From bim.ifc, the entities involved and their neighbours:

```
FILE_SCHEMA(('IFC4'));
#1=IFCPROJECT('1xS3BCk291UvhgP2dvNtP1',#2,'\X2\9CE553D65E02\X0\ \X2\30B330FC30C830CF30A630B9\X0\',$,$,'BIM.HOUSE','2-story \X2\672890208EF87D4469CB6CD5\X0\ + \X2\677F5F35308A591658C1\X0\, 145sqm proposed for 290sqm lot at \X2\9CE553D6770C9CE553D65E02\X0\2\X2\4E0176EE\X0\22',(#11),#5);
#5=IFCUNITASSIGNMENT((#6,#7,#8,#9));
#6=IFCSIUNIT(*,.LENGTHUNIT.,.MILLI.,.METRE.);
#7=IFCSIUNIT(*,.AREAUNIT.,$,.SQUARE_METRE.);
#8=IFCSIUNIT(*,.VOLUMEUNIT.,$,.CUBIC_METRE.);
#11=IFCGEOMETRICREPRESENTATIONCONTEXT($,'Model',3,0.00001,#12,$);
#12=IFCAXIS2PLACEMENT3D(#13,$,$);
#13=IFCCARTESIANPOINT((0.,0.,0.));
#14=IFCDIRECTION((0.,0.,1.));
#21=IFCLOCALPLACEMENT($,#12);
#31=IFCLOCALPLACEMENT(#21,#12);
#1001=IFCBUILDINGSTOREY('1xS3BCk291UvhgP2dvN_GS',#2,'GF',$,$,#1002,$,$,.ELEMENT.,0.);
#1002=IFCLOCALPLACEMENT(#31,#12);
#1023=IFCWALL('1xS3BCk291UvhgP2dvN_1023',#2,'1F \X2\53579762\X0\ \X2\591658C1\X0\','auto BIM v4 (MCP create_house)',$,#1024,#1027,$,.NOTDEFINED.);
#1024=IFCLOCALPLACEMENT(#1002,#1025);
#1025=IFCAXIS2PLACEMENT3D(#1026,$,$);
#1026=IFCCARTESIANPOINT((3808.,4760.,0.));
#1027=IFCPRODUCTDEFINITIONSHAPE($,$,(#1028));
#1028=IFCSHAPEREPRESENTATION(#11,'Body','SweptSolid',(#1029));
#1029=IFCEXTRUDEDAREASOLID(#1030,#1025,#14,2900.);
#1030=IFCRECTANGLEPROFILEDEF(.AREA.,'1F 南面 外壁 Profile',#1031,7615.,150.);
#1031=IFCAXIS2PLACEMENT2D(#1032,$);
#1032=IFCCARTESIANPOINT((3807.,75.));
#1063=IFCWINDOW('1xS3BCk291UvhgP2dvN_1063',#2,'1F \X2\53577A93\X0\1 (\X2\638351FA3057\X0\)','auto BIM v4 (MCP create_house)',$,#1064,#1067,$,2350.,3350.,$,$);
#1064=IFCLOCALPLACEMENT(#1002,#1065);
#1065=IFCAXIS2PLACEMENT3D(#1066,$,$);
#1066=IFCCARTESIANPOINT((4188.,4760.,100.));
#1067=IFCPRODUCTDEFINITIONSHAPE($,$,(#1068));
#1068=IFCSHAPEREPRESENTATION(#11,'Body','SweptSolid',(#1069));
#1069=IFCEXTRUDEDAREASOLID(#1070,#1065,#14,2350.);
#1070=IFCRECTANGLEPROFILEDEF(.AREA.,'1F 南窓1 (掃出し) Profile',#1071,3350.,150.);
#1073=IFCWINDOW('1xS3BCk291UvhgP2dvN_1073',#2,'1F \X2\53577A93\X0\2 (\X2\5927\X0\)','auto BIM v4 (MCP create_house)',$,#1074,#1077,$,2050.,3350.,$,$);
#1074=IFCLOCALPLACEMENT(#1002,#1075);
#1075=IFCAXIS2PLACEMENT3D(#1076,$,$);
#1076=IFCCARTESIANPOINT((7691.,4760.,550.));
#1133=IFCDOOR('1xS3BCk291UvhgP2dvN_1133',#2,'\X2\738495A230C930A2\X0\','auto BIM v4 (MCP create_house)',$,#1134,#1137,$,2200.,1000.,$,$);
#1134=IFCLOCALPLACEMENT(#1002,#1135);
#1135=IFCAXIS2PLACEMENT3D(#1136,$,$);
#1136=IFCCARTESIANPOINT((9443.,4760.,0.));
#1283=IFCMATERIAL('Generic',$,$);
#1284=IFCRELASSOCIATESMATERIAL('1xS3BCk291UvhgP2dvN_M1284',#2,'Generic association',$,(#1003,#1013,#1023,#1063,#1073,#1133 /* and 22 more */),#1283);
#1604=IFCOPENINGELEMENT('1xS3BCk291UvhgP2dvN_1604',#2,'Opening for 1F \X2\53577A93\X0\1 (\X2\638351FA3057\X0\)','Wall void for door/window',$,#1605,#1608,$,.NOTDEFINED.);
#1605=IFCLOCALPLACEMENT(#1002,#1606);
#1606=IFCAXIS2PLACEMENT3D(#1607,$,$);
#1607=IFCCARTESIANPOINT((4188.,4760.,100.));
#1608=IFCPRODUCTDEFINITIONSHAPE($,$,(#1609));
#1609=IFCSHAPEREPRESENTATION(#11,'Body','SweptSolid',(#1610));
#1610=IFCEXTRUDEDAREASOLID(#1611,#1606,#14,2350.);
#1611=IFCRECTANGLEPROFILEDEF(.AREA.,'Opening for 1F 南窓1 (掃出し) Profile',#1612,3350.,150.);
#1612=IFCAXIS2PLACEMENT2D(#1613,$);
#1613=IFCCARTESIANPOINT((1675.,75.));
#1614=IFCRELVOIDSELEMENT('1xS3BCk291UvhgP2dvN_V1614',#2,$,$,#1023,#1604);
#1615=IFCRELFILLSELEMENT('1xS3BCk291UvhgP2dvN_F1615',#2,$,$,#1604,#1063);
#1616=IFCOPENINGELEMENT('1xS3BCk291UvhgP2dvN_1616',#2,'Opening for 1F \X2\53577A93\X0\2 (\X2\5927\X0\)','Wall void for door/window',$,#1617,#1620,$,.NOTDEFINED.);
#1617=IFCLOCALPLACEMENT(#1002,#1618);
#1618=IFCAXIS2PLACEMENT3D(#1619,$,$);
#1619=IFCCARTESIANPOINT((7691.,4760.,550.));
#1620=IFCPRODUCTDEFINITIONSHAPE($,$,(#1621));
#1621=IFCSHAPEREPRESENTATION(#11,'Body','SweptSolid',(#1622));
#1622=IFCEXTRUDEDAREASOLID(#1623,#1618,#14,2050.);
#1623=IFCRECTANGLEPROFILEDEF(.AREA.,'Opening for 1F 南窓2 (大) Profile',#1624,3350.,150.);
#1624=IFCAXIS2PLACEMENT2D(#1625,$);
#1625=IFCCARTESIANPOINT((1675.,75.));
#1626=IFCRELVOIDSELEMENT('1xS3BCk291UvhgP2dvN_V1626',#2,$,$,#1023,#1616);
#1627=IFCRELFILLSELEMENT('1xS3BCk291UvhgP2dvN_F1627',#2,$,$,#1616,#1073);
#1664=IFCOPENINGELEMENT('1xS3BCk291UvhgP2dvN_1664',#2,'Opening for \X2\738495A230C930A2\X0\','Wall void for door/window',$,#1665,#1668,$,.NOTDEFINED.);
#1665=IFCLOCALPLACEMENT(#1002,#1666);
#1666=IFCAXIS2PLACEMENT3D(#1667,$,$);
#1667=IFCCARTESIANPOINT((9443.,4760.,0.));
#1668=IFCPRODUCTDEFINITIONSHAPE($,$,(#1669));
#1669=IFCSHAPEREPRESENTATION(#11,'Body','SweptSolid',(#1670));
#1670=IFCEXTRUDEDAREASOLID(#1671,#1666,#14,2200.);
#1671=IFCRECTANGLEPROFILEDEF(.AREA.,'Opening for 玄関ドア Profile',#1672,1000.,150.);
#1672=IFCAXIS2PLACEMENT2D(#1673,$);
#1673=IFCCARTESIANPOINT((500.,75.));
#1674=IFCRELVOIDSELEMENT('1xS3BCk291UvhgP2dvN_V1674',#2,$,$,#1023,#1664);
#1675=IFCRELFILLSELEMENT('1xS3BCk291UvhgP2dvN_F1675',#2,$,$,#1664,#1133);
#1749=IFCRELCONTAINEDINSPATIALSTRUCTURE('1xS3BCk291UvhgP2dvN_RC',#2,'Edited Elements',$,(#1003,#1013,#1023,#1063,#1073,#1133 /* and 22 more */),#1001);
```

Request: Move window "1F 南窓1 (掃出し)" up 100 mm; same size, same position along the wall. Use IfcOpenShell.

```python
import numpy as np
import ifcopenshell
import ifcopenshell.api.geometry
import ifcopenshell.util.placement
import ifcopenshell.util.unit

model = ifcopenshell.open("bim.ifc")
unit_scale = ifcopenshell.util.unit.calculate_unit_scale(model)

window = model.by_guid("1xS3BCk291UvhgP2dvN_1063")
opening = window.FillsVoids[0].RelatingOpeningElement
dz = 100.0

shift = np.array([0.0, 0.0, dz])
# The window is not placed relative to its opening, so move both.
for product in (opening, window):
    matrix = ifcopenshell.util.placement.get_local_placement(product.ObjectPlacement)
    matrix[:3, 3] += shift
    ifcopenshell.api.geometry.edit_object_placement(model, product=product, matrix=matrix, is_si=False)

print(f"moved by {dz * unit_scale:+.3f} m")

model.write("bim_v2.ifc")
```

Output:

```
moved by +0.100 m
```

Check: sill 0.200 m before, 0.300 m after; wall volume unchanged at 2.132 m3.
